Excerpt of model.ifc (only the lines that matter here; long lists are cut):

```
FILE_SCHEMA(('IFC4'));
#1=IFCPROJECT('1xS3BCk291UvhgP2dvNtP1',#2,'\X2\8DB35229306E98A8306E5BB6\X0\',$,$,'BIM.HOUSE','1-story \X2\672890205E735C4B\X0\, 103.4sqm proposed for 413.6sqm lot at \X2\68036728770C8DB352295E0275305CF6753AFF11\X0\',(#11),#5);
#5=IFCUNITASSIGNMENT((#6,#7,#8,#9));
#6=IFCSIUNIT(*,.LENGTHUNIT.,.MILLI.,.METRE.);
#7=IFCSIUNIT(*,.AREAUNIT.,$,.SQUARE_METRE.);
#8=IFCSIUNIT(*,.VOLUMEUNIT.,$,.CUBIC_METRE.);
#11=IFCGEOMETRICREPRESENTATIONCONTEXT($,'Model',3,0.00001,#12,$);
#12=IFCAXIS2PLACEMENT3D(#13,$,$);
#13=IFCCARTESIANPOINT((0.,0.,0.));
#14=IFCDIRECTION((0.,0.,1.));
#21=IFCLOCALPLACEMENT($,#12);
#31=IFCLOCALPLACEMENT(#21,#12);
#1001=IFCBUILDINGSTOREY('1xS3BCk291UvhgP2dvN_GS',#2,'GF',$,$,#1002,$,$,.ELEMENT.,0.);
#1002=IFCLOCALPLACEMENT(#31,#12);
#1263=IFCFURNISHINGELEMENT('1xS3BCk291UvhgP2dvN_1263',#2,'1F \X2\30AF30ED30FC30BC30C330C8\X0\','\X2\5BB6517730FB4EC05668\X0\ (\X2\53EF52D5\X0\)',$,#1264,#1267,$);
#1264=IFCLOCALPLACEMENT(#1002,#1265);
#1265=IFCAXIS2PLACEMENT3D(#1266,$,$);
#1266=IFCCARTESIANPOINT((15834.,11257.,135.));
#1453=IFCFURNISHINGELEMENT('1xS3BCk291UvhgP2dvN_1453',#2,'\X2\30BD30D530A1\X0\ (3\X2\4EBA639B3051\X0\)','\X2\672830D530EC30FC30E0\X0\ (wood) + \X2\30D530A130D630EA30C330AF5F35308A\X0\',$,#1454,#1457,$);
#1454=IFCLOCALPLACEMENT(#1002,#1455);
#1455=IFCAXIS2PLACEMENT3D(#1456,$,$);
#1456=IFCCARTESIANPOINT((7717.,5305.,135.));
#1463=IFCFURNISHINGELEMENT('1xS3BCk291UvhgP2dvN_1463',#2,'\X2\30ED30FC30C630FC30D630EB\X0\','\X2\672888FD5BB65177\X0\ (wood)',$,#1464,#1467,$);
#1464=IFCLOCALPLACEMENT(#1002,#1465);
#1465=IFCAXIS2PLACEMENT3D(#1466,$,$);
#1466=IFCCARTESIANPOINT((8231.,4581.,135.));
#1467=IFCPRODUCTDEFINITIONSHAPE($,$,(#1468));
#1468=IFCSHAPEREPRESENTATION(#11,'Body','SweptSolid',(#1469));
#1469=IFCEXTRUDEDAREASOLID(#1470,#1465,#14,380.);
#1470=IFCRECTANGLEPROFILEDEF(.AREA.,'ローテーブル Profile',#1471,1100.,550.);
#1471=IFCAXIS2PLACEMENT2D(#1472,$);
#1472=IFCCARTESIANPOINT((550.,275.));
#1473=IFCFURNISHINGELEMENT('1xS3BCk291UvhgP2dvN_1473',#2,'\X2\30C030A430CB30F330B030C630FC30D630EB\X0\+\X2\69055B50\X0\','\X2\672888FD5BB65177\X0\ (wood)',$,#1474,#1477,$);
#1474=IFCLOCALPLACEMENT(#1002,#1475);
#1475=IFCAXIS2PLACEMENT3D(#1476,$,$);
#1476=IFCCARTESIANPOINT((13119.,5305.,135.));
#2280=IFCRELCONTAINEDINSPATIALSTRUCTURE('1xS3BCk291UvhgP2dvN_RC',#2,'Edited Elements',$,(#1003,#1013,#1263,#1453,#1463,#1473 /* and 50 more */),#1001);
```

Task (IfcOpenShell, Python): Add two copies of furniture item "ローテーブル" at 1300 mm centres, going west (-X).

```python
import numpy as np
import ifcopenshell
import ifcopenshell.api.geometry
import ifcopenshell.api.root
import ifcopenshell.util.element
import ifcopenshell.util.placement
import ifcopenshell.util.unit

model = ifcopenshell.open("model.ifc")
unit_scale = ifcopenshell.util.unit.calculate_unit_scale(model)


def reuse_history(source, copy):
    """copy_class also copies each property set's owner history, people and application; keep the originals."""
    for rel in copy.IsDefinedBy:
        if rel.is_a("IfcRelDefinesByProperties") and (history := rel.RelatingPropertyDefinition.OwnerHistory):
            rel.RelatingPropertyDefinition.OwnerHistory = source.OwnerHistory
            ifcopenshell.util.element.remove_deep2(model, history)


source = model.by_guid("1xS3BCk291UvhgP2dvN_1463")
base = ifcopenshell.util.placement.get_local_placement(source.ObjectPlacement)
step = np.array([-1.0, 0.0, 0.0]) * 1.3 / unit_scale

for i in range(1, 3):
    copy = ifcopenshell.api.root.copy_class(model, product=source)
    copy.Representation = ifcopenshell.util.element.copy_deep(
        model, source.Representation, exclude=["IfcGeometricRepresentationContext", "IfcRepresentationMap"]
    )
    reuse_history(source, copy)
    matrix = base.copy()
    matrix[:3, 3] += i * step
    print("added at", matrix[:3, 3].round(3) + 0.0)
    ifcopenshell.api.geometry.edit_object_placement(model, product=copy, matrix=matrix, is_si=False)

model.write("model-out.ifc")
```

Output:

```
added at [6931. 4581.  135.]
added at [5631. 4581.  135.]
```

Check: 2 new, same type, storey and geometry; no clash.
